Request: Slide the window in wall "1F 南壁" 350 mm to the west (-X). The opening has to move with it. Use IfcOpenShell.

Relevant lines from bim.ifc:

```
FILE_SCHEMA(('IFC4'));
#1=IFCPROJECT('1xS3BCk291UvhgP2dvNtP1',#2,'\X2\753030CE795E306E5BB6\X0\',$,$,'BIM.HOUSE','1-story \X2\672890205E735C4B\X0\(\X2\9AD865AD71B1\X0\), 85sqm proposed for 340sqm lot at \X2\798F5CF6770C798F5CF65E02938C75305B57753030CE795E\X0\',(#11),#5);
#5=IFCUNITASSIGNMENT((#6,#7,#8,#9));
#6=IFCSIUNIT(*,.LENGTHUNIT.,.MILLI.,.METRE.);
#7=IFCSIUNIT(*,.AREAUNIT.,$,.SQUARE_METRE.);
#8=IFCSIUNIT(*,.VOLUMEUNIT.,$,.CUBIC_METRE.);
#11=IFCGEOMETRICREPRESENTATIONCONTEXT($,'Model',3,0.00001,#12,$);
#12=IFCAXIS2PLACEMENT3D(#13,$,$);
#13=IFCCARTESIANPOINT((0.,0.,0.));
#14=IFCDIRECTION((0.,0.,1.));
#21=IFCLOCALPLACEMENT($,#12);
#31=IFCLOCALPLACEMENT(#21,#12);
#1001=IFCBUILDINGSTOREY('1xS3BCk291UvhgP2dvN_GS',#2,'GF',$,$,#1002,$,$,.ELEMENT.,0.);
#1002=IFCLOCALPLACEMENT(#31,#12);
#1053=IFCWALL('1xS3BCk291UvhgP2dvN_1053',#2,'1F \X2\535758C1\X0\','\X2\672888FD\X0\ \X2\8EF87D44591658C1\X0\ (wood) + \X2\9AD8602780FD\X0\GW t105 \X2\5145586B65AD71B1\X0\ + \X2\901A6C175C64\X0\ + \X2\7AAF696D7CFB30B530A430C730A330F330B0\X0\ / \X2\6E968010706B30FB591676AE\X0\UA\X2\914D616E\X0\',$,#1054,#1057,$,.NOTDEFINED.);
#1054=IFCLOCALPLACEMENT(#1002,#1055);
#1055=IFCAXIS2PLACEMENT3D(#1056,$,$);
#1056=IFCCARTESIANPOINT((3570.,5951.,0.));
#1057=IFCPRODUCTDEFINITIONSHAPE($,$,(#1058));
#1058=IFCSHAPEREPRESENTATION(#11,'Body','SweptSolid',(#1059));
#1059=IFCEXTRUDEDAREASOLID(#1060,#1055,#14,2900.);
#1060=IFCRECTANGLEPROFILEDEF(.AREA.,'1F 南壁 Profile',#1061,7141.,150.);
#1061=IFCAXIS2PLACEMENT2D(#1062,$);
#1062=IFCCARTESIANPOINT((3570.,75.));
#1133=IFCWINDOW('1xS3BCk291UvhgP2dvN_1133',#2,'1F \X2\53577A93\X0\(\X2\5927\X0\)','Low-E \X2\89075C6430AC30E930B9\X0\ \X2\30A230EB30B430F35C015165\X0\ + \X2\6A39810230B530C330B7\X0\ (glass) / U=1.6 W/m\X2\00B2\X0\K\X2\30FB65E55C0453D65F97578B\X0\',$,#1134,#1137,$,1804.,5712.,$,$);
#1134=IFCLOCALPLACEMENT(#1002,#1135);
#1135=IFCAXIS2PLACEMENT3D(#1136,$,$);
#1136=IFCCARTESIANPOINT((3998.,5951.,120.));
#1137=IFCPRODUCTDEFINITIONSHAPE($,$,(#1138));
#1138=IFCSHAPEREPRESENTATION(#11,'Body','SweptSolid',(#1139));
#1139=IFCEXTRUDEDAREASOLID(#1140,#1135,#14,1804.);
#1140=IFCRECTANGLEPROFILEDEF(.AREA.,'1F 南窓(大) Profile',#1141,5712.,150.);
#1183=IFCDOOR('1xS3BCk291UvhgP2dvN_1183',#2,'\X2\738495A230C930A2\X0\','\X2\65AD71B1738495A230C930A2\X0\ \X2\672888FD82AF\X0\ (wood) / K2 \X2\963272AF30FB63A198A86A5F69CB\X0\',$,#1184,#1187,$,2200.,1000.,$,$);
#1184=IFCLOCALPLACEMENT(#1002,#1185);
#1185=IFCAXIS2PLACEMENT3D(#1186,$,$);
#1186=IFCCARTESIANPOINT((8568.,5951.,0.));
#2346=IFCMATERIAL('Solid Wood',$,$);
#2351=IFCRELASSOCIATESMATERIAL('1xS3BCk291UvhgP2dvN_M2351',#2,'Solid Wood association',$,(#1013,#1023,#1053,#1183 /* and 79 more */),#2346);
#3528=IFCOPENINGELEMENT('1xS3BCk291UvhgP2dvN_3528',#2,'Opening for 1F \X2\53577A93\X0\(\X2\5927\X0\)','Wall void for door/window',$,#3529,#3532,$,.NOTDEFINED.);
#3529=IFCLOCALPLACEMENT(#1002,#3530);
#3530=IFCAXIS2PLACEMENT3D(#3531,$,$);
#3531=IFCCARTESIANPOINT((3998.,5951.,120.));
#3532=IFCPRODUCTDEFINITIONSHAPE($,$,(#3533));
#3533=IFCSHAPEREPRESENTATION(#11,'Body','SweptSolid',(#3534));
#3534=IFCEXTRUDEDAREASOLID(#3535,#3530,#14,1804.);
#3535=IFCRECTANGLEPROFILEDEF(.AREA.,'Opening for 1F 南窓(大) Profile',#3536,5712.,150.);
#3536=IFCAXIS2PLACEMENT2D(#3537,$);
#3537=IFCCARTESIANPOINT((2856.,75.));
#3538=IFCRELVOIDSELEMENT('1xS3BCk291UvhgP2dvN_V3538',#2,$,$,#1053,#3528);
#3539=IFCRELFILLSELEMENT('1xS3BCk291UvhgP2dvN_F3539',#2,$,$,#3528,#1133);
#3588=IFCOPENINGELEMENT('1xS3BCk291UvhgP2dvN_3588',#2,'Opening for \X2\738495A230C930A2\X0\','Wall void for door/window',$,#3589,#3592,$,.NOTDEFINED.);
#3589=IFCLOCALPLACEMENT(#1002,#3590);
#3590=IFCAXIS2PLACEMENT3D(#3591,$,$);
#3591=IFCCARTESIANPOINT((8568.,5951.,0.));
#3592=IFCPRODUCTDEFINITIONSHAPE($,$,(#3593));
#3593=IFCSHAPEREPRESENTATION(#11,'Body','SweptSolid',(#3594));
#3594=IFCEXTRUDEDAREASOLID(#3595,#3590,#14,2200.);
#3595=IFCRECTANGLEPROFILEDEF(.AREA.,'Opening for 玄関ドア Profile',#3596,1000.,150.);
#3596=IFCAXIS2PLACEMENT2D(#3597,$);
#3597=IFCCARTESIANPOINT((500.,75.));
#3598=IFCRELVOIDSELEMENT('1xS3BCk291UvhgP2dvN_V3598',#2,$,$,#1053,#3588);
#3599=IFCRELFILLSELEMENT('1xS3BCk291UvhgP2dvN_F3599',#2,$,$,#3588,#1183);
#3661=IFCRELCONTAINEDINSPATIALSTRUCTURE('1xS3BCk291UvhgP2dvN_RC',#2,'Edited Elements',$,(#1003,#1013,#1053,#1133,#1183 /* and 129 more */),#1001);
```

```python
import ifcopenshell
import ifcopenshell.api.geometry
import ifcopenshell.util.placement
import ifcopenshell.util.unit

model = ifcopenshell.open("bim.ifc")
unit_scale = ifcopenshell.util.unit.calculate_unit_scale(model)

window = model.by_id(1133)
opening = window.FillsVoids[0].RelatingOpeningElement
wall = opening.VoidsElements[0].RelatingBuildingElement

wall_matrix = ifcopenshell.util.placement.get_local_placement(wall.ObjectPlacement)
shift = wall_matrix[:3, 0] * -0.35 / unit_scale
before = ifcopenshell.util.placement.get_local_placement(window.ObjectPlacement)[:3, 3].copy()

# The window is not placed relative to its opening, so move both.
for product in (opening, window):
    matrix = ifcopenshell.util.placement.get_local_placement(product.ObjectPlacement)
    matrix[:3, 3] += shift
    ifcopenshell.api.geometry.edit_object_placement(model, product=product, matrix=matrix, is_si=False)

after = ifcopenshell.util.placement.get_local_placement(window.ObjectPlacement)[:3, 3]
print("window moved by", (after - before).round(3) + 0.0)

model.write("bim_edited.ifc")
```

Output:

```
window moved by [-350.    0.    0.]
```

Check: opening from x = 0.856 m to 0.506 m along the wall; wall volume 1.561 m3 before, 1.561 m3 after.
